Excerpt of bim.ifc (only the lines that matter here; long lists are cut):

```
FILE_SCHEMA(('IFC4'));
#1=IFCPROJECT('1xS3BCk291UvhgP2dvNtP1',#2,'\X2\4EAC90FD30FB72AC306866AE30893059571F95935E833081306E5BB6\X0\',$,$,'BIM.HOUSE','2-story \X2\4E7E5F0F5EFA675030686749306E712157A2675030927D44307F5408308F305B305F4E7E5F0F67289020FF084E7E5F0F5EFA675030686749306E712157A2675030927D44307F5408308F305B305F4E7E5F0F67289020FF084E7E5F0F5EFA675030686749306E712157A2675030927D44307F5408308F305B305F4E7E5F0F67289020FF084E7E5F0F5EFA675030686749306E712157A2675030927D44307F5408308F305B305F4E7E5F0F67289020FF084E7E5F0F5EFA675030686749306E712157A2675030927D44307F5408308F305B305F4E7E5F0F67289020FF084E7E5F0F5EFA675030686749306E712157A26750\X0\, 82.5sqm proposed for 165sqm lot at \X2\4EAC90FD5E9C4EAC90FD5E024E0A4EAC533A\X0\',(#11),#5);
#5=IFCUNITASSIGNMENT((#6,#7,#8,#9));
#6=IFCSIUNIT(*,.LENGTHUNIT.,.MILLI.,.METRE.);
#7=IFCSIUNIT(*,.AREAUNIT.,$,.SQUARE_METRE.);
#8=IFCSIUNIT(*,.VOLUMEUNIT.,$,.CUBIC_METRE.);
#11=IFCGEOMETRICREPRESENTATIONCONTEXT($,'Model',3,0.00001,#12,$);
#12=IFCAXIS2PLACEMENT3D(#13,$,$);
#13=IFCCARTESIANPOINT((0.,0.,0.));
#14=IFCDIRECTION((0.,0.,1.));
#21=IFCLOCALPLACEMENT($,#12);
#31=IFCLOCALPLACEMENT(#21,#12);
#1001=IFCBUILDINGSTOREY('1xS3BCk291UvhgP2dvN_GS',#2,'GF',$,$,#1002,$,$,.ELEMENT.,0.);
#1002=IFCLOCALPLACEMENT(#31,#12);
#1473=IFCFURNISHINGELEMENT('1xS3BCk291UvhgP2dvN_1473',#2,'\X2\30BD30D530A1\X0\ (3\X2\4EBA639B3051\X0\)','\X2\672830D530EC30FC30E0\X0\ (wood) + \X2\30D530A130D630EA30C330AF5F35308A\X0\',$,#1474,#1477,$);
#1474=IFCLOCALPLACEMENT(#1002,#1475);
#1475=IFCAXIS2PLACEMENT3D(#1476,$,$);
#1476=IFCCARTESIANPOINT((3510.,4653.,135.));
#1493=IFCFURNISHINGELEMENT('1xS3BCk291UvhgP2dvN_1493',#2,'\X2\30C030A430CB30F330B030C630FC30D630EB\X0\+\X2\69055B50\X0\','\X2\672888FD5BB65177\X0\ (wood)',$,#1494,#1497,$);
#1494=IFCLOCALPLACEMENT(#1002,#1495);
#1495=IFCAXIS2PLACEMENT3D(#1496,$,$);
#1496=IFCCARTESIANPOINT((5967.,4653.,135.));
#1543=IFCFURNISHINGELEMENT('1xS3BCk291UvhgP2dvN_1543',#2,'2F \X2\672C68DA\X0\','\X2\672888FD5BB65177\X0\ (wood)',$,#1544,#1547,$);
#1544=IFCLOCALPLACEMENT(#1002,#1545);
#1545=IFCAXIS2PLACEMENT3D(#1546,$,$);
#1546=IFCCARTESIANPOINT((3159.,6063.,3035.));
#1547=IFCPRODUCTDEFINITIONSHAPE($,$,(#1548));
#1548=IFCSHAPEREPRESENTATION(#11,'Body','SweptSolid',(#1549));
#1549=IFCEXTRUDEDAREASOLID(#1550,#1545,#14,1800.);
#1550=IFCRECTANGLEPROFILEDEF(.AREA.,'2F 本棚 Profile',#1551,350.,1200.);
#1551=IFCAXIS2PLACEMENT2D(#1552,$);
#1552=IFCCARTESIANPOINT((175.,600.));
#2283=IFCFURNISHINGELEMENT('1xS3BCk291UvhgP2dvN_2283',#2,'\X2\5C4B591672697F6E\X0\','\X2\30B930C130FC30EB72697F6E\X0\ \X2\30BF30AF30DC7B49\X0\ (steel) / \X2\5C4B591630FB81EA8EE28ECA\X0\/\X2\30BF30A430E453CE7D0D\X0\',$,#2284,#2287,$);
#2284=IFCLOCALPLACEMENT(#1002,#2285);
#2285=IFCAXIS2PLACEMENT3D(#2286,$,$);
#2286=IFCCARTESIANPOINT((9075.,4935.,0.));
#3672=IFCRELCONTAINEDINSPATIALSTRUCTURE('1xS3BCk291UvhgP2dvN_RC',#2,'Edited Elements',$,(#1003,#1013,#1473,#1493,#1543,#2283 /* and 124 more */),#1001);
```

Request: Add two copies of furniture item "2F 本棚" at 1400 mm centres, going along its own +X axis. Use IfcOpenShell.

```python
import ifcopenshell
import ifcopenshell.api.geometry
import ifcopenshell.api.root
import ifcopenshell.util.element
import ifcopenshell.util.placement
import ifcopenshell.util.unit

model = ifcopenshell.open("bim.ifc")
unit_scale = ifcopenshell.util.unit.calculate_unit_scale(model)


def reuse_history(source, copy):
    """copy_class also copies each property set's owner history, people and application; keep the originals."""
    for rel in copy.IsDefinedBy:
        if rel.is_a("IfcRelDefinesByProperties") and (history := rel.RelatingPropertyDefinition.OwnerHistory):
            rel.RelatingPropertyDefinition.OwnerHistory = source.OwnerHistory
            ifcopenshell.util.element.remove_deep2(model, history)


source = model.by_id(1543)
base = ifcopenshell.util.placement.get_local_placement(source.ObjectPlacement)
step = base[:3, 0] * 1.4 / unit_scale

for i in range(1, 3):
    copy = ifcopenshell.api.root.copy_class(model, product=source)
    copy.Representation = ifcopenshell.util.element.copy_deep(
        model, source.Representation, exclude=["IfcGeometricRepresentationContext", "IfcRepresentationMap"]
    )
    reuse_history(source, copy)
    matrix = base.copy()
    matrix[:3, 3] += i * step
    print("added at", matrix[:3, 3].round(3) + 0.0)
    ifcopenshell.api.geometry.edit_object_placement(model, product=copy, matrix=matrix, is_si=False)

model.write("bim_v2.ifc")
```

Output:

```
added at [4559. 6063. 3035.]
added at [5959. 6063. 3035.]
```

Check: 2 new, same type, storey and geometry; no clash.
